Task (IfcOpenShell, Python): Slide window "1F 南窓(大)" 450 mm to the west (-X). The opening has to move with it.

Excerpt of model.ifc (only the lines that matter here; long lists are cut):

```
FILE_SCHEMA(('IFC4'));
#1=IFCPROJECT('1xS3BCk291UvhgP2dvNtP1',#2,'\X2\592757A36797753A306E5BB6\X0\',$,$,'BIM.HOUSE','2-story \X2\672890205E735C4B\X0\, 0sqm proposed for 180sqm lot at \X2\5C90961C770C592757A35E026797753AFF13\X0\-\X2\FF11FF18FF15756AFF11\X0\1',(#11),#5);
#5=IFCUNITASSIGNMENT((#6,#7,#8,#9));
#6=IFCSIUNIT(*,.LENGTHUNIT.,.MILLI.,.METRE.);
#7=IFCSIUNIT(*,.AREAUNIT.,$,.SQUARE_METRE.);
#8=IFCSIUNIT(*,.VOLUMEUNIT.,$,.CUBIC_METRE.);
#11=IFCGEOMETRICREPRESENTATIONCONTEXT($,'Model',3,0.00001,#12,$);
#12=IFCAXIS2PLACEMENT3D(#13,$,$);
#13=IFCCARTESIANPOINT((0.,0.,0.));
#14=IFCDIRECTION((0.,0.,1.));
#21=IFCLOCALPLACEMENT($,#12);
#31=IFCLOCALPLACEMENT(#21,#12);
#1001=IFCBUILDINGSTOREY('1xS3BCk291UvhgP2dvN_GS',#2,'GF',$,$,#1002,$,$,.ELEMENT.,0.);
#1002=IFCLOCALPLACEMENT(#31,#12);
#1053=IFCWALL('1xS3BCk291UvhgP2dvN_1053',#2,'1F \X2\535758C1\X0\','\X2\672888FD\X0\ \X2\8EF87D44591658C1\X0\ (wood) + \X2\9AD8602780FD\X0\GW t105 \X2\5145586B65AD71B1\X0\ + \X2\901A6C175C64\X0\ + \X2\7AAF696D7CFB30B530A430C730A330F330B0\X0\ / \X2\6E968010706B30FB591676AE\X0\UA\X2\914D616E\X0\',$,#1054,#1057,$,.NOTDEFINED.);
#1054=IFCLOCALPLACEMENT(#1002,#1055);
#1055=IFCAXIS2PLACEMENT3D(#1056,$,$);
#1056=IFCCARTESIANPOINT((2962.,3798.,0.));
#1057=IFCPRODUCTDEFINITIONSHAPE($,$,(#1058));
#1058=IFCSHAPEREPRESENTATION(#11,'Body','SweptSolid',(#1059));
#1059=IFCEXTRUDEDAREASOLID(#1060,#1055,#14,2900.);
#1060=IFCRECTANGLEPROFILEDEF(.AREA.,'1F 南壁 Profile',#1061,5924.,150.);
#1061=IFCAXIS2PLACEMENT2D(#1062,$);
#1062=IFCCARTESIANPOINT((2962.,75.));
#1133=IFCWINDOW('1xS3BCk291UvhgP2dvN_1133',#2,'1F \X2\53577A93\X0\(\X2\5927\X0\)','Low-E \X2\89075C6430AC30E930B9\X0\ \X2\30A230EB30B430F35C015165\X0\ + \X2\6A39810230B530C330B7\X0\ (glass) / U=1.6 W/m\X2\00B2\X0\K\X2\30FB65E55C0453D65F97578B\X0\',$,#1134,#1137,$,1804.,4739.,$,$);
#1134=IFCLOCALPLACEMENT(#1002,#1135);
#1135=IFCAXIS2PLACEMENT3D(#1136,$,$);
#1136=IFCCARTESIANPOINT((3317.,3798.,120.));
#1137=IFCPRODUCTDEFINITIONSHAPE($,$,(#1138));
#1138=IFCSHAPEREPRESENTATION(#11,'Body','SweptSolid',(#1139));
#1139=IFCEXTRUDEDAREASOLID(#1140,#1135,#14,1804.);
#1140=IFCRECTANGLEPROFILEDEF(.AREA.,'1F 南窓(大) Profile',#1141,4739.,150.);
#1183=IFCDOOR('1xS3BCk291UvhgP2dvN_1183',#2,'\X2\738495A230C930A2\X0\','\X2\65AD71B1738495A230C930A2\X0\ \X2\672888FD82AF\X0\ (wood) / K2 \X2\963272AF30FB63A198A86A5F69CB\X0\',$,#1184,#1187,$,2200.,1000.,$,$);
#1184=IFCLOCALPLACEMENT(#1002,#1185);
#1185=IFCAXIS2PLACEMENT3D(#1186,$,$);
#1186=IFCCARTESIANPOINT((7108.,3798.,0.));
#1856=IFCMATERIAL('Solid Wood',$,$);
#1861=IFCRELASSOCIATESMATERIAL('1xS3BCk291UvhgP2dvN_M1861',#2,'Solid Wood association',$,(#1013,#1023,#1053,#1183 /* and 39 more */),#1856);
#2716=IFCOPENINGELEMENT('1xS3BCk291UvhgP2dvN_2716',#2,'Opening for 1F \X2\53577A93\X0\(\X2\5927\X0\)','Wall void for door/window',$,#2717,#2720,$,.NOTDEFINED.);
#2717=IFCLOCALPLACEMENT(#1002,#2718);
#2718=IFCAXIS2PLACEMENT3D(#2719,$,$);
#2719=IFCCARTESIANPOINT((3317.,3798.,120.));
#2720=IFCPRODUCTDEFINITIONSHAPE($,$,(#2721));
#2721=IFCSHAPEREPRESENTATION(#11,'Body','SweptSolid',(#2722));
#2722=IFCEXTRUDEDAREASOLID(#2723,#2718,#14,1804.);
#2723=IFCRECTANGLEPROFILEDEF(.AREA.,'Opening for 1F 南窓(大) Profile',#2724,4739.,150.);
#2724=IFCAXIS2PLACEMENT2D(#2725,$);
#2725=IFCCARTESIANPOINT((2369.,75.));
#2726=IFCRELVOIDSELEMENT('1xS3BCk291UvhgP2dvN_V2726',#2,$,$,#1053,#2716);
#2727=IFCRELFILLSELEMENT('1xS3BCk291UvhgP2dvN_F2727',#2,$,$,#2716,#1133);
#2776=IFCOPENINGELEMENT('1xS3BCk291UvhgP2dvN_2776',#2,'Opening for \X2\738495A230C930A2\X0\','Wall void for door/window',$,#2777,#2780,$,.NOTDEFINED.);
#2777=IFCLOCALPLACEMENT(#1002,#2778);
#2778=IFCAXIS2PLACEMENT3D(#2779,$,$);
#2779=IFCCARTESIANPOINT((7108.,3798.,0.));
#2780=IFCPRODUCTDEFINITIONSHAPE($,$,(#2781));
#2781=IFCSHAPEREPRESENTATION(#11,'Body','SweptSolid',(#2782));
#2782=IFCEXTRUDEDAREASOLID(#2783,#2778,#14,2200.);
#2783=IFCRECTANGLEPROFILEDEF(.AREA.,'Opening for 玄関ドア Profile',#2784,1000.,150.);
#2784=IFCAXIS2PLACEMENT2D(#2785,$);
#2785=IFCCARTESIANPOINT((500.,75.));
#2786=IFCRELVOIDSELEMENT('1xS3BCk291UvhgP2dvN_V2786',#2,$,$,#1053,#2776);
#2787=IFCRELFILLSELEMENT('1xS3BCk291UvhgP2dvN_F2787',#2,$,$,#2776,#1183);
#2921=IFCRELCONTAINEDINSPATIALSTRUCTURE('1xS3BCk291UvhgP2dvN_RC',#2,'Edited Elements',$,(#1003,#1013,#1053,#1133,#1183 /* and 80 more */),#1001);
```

```python
import ifcopenshell
import ifcopenshell.api.geometry
import ifcopenshell.util.placement
import ifcopenshell.util.unit

model = ifcopenshell.open("model.ifc")
unit_scale = ifcopenshell.util.unit.calculate_unit_scale(model)

window = model.by_guid("1xS3BCk291UvhgP2dvN_1133")
opening = window.FillsVoids[0].RelatingOpeningElement
wall = opening.VoidsElements[0].RelatingBuildingElement

wall_matrix = ifcopenshell.util.placement.get_local_placement(wall.ObjectPlacement)
shift = wall_matrix[:3, 0] * -0.45 / unit_scale
before = ifcopenshell.util.placement.get_local_placement(window.ObjectPlacement)[:3, 3].copy()

# The window is not placed relative to its opening, so move both.
for product in (opening, window):
    matrix = ifcopenshell.util.placement.get_local_placement(product.ObjectPlacement)
    matrix[:3, 3] += shift
    ifcopenshell.api.geometry.edit_object_placement(model, product=product, matrix=matrix, is_si=False)

after = ifcopenshell.util.placement.get_local_placement(window.ObjectPlacement)[:3, 3]
print("window moved by", (after - before).round(3) + 0.0)

model.write("model-out.ifc")
```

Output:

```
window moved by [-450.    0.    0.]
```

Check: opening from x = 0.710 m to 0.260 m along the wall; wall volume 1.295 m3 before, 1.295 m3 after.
